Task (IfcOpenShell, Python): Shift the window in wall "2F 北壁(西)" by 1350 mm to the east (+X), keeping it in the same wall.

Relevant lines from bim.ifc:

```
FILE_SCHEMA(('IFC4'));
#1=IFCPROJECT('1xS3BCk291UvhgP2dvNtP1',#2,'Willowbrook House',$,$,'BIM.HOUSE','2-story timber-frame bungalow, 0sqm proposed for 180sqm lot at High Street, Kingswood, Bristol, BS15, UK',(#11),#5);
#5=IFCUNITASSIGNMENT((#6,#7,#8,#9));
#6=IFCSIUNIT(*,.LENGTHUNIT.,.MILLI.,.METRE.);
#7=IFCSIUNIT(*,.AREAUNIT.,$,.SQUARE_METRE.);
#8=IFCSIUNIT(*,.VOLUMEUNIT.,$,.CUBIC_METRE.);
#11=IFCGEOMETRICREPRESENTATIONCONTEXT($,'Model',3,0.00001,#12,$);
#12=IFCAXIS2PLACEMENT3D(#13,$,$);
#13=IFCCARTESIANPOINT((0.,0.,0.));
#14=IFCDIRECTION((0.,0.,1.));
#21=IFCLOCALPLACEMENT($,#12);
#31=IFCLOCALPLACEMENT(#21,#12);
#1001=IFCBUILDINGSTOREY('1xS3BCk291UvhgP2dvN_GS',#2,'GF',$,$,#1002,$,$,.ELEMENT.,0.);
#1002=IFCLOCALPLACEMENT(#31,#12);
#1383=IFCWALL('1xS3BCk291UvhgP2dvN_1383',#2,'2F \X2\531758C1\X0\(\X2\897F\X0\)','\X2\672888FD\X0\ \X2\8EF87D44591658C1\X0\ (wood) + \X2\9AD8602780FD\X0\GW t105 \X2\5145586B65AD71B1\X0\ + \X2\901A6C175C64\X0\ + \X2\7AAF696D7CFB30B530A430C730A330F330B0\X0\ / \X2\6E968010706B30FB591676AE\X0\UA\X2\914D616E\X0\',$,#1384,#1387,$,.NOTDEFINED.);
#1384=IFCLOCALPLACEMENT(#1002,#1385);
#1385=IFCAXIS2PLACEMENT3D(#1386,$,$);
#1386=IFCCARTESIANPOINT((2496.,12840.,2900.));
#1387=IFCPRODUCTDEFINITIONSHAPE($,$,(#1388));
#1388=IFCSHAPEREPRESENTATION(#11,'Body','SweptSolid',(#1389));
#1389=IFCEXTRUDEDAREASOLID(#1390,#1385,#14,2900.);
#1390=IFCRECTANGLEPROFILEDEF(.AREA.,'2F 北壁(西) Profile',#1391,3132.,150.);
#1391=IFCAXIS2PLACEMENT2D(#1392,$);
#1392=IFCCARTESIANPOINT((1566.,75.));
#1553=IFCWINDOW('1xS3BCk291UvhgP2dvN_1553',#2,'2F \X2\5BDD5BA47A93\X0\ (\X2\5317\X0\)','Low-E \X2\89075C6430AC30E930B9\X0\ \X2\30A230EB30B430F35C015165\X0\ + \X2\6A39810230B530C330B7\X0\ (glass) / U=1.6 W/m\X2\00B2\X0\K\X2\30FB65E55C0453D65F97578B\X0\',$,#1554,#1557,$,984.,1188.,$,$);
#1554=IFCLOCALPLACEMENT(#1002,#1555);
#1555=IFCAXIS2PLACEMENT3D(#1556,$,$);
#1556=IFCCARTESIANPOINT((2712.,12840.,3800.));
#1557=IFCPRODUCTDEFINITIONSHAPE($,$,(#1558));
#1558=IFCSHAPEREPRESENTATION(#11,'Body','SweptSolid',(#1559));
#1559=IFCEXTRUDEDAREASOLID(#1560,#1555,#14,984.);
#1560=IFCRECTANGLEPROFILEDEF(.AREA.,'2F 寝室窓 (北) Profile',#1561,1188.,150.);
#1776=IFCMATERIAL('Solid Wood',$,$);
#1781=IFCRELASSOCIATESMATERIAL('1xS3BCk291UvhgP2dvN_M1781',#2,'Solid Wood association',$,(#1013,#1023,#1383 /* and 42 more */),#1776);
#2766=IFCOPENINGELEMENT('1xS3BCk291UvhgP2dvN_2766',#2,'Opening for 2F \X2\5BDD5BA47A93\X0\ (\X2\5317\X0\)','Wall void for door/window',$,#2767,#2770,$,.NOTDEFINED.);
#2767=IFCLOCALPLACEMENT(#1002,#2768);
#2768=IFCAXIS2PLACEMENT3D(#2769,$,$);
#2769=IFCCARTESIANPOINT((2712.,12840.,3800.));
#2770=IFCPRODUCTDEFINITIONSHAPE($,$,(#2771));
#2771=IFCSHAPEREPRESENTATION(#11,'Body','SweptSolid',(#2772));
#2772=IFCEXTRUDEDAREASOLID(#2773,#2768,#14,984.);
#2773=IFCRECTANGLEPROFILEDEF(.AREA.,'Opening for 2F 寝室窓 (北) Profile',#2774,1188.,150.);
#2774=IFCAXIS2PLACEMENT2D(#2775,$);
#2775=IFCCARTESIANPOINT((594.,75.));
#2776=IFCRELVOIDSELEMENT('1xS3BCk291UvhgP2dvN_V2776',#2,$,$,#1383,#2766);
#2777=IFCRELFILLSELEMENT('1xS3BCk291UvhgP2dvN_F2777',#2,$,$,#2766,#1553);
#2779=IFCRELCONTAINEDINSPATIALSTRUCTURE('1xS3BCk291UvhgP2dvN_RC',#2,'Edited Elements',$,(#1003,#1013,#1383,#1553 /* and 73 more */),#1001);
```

```python
import ifcopenshell
import ifcopenshell.api.geometry
import ifcopenshell.util.placement

model = ifcopenshell.open("bim.ifc")

window = model.by_guid("1xS3BCk291UvhgP2dvN_1553")
opening = window.FillsVoids[0].RelatingOpeningElement
wall = opening.VoidsElements[0].RelatingBuildingElement

wall_matrix = ifcopenshell.util.placement.get_local_placement(wall.ObjectPlacement)
shift = wall_matrix[:3, 0] * 1350.0
before = ifcopenshell.util.placement.get_local_placement(window.ObjectPlacement)[:3, 3].copy()

# The window is not placed relative to its opening, so move both.
for product in (opening, window):
    matrix = ifcopenshell.util.placement.get_local_placement(product.ObjectPlacement)
    matrix[:3, 3] += shift
    ifcopenshell.api.geometry.edit_object_placement(model, product=product, matrix=matrix, is_si=False)

after = ifcopenshell.util.placement.get_local_placement(window.ObjectPlacement)[:3, 3]
print("window moved by", (after - before).round(3) + 0.0)

model.write("bim-out.ifc")
```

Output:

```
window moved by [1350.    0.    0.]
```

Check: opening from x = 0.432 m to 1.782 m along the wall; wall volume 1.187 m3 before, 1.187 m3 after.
